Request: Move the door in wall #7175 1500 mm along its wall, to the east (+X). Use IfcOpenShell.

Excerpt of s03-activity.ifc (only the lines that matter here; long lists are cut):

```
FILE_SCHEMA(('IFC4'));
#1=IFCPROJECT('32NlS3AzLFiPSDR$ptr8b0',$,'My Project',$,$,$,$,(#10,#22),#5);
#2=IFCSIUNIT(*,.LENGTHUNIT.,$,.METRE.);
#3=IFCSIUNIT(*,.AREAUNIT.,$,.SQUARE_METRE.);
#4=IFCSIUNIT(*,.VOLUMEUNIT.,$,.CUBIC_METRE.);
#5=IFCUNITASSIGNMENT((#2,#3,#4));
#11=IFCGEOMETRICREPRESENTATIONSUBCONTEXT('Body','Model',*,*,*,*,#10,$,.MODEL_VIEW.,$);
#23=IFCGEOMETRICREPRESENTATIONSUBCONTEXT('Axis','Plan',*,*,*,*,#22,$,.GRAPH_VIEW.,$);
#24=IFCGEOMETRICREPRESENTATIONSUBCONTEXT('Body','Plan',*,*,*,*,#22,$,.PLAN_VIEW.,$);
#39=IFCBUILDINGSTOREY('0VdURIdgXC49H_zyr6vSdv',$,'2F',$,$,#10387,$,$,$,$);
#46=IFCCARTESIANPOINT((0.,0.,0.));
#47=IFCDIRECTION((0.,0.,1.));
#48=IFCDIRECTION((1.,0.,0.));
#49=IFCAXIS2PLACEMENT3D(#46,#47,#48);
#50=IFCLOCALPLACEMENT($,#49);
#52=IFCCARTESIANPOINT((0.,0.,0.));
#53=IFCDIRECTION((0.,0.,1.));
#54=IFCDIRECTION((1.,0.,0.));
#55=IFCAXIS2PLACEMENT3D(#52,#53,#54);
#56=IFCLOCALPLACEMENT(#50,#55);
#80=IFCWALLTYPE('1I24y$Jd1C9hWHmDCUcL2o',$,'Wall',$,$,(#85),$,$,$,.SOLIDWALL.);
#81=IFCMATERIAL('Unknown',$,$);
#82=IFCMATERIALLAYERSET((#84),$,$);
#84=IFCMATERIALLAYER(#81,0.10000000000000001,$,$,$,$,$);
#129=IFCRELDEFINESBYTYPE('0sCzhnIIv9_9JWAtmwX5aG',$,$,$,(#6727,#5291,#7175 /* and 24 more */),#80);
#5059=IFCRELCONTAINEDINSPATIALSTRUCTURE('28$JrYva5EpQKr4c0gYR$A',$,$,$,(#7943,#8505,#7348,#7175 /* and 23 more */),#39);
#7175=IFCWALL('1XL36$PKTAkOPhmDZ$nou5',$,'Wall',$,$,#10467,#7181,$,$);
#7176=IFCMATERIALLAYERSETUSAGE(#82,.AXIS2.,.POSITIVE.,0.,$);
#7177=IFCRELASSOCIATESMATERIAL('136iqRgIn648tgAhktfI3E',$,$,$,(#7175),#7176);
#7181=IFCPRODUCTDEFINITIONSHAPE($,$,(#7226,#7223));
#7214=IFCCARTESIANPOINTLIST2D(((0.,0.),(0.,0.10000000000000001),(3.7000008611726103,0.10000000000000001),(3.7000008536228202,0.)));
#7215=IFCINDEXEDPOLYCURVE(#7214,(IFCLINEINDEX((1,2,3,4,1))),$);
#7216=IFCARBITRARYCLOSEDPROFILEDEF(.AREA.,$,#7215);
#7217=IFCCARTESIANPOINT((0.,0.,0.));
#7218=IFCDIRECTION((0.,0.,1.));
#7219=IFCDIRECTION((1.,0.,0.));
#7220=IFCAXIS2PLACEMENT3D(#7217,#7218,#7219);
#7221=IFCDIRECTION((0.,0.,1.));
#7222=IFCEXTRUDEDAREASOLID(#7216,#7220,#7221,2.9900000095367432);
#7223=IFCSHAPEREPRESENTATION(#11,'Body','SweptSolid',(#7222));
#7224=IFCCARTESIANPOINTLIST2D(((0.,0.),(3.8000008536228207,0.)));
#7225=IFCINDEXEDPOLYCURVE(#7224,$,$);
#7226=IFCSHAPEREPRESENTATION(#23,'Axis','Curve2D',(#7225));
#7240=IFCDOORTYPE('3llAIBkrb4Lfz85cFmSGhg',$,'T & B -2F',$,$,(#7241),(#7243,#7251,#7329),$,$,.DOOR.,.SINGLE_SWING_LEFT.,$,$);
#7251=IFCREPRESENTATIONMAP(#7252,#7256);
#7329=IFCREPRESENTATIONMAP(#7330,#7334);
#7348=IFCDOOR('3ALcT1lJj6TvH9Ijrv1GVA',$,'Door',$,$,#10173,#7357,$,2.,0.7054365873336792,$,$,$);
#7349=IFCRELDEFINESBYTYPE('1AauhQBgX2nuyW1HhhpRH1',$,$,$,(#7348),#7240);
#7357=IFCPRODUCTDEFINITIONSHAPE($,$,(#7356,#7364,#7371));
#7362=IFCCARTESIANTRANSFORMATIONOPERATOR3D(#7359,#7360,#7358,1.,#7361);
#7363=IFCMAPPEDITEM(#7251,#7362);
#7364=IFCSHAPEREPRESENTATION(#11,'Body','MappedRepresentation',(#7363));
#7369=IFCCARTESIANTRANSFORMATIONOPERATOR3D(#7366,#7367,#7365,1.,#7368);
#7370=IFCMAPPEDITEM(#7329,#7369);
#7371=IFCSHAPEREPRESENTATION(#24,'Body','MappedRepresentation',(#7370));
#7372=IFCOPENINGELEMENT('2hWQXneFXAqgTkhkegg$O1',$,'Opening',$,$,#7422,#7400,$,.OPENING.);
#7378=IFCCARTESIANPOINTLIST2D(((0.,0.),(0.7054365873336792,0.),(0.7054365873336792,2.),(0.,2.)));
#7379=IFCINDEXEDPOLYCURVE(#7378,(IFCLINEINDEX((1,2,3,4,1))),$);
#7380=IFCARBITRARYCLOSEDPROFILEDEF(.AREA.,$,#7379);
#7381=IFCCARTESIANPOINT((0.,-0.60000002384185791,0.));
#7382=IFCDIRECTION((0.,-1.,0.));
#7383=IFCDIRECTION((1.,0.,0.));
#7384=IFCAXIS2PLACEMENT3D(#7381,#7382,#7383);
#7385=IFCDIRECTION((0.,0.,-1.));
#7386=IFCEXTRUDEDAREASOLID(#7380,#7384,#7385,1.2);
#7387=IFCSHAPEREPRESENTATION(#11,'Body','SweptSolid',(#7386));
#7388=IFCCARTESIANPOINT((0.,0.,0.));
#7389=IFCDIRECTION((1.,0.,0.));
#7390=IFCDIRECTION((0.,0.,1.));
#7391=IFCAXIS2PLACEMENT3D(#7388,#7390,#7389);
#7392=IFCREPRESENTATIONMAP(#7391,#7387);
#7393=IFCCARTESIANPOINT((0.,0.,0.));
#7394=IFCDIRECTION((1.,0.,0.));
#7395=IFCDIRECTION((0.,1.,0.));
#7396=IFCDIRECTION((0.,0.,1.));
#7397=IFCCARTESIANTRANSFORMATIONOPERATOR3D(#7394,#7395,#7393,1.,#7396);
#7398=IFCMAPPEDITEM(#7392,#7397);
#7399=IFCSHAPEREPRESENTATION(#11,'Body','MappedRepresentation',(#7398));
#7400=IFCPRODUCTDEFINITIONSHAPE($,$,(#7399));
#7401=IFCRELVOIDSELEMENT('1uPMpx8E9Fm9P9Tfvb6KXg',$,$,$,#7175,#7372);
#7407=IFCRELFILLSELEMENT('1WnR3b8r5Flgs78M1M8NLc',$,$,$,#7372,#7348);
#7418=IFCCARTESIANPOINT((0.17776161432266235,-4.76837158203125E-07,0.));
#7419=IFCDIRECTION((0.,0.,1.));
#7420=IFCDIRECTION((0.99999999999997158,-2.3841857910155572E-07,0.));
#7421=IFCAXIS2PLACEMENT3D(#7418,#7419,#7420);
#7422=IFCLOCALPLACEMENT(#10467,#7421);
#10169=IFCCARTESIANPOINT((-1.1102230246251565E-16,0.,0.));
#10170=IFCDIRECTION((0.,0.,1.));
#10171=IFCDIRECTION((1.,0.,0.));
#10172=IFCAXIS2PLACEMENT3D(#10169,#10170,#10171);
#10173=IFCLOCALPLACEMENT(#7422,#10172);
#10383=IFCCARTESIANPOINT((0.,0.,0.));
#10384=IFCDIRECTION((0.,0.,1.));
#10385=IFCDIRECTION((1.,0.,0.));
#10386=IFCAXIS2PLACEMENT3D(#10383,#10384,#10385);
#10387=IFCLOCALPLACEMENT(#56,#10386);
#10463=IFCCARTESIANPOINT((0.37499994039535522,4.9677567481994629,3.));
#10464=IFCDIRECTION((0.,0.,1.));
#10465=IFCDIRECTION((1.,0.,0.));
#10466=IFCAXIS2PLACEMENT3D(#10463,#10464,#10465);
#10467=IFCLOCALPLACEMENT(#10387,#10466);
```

```python
import ifcopenshell
import ifcopenshell.api.geometry
import ifcopenshell.util.placement

model = ifcopenshell.open("s03-activity.ifc")

door = model.by_guid("3ALcT1lJj6TvH9Ijrv1GVA")
opening = door.FillsVoids[0].RelatingOpeningElement
wall = opening.VoidsElements[0].RelatingBuildingElement

wall_matrix = ifcopenshell.util.placement.get_local_placement(wall.ObjectPlacement)
shift = wall_matrix[:3, 0] * 1.5
before = ifcopenshell.util.placement.get_local_placement(door.ObjectPlacement)[:3, 3].copy()

# The door is placed relative to its opening, so it follows when the opening moves.
matrix = ifcopenshell.util.placement.get_local_placement(opening.ObjectPlacement)
matrix[:3, 3] += shift
ifcopenshell.api.geometry.edit_object_placement(
    model, product=opening, matrix=matrix, is_si=False, should_transform_children=True
)

after = ifcopenshell.util.placement.get_local_placement(door.ObjectPlacement)[:3, 3]
print("door moved by", (after - before).round(3) + 0.0)

model.write("s03-activity-out.ifc")
```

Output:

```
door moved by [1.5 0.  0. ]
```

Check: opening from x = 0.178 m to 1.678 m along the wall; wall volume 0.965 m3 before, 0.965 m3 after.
